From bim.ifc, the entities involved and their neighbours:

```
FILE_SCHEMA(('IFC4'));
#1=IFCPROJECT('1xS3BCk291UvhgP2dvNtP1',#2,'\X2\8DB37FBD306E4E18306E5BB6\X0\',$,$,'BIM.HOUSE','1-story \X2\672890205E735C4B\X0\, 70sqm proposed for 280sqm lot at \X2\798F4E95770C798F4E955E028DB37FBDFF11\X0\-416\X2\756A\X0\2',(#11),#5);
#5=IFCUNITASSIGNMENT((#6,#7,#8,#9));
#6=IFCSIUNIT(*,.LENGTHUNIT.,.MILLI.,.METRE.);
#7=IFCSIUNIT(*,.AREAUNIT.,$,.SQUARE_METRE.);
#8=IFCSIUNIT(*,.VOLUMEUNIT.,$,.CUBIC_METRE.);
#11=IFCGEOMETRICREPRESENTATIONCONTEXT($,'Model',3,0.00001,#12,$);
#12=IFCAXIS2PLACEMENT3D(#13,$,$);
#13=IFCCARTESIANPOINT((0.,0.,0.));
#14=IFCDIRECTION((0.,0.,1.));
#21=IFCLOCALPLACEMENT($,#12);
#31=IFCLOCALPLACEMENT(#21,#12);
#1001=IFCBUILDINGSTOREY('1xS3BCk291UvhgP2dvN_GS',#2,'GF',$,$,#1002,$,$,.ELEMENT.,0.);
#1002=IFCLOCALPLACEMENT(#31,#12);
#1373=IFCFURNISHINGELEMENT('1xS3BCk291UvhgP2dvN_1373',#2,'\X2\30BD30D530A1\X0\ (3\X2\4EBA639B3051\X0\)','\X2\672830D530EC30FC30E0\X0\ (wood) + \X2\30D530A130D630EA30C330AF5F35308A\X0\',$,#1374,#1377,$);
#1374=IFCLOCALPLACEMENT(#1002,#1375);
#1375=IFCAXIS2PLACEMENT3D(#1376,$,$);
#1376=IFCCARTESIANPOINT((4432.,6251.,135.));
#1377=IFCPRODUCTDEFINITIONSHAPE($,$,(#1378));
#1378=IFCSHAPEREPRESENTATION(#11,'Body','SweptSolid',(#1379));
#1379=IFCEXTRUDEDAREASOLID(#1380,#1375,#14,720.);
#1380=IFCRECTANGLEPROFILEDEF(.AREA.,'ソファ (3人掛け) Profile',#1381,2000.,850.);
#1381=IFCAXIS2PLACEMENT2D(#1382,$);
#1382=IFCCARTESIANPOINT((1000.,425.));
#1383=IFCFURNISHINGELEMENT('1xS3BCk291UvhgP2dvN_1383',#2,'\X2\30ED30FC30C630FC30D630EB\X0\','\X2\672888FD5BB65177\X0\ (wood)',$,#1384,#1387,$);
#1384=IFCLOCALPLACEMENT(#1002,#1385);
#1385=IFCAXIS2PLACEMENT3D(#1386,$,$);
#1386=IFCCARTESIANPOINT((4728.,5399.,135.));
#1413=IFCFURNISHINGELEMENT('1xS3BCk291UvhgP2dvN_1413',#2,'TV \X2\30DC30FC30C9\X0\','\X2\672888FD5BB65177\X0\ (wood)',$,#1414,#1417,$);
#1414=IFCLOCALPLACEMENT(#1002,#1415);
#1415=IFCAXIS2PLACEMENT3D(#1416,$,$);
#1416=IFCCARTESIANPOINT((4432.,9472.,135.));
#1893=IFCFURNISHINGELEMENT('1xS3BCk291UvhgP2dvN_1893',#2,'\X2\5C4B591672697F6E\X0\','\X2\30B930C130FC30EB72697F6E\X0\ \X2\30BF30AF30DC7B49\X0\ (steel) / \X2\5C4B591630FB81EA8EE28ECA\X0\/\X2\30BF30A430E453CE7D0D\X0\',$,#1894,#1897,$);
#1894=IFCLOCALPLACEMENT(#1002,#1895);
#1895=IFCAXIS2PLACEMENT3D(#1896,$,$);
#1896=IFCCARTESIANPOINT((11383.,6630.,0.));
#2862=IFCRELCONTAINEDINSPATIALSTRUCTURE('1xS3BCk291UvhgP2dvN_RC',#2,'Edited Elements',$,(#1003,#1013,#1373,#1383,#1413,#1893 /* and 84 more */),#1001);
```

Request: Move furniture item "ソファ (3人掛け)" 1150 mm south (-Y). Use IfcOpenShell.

```python
import ifcopenshell
import ifcopenshell.api.geometry
import ifcopenshell.util.placement

model = ifcopenshell.open("bim.ifc")

item = model.by_guid("1xS3BCk291UvhgP2dvN_1373")
matrix = ifcopenshell.util.placement.get_local_placement(item.ObjectPlacement)
matrix[1, 3] -= 1150.0
ifcopenshell.api.geometry.edit_object_placement(model, product=item, matrix=matrix, is_si=False)

print(ifcopenshell.util.placement.get_local_placement(item.ObjectPlacement).round(3) + 0.0)

model.write("bim-out.ifc")
```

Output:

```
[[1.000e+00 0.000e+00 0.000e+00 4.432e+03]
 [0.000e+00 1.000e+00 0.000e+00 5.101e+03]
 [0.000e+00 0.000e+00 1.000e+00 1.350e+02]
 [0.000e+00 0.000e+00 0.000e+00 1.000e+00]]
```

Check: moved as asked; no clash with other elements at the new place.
